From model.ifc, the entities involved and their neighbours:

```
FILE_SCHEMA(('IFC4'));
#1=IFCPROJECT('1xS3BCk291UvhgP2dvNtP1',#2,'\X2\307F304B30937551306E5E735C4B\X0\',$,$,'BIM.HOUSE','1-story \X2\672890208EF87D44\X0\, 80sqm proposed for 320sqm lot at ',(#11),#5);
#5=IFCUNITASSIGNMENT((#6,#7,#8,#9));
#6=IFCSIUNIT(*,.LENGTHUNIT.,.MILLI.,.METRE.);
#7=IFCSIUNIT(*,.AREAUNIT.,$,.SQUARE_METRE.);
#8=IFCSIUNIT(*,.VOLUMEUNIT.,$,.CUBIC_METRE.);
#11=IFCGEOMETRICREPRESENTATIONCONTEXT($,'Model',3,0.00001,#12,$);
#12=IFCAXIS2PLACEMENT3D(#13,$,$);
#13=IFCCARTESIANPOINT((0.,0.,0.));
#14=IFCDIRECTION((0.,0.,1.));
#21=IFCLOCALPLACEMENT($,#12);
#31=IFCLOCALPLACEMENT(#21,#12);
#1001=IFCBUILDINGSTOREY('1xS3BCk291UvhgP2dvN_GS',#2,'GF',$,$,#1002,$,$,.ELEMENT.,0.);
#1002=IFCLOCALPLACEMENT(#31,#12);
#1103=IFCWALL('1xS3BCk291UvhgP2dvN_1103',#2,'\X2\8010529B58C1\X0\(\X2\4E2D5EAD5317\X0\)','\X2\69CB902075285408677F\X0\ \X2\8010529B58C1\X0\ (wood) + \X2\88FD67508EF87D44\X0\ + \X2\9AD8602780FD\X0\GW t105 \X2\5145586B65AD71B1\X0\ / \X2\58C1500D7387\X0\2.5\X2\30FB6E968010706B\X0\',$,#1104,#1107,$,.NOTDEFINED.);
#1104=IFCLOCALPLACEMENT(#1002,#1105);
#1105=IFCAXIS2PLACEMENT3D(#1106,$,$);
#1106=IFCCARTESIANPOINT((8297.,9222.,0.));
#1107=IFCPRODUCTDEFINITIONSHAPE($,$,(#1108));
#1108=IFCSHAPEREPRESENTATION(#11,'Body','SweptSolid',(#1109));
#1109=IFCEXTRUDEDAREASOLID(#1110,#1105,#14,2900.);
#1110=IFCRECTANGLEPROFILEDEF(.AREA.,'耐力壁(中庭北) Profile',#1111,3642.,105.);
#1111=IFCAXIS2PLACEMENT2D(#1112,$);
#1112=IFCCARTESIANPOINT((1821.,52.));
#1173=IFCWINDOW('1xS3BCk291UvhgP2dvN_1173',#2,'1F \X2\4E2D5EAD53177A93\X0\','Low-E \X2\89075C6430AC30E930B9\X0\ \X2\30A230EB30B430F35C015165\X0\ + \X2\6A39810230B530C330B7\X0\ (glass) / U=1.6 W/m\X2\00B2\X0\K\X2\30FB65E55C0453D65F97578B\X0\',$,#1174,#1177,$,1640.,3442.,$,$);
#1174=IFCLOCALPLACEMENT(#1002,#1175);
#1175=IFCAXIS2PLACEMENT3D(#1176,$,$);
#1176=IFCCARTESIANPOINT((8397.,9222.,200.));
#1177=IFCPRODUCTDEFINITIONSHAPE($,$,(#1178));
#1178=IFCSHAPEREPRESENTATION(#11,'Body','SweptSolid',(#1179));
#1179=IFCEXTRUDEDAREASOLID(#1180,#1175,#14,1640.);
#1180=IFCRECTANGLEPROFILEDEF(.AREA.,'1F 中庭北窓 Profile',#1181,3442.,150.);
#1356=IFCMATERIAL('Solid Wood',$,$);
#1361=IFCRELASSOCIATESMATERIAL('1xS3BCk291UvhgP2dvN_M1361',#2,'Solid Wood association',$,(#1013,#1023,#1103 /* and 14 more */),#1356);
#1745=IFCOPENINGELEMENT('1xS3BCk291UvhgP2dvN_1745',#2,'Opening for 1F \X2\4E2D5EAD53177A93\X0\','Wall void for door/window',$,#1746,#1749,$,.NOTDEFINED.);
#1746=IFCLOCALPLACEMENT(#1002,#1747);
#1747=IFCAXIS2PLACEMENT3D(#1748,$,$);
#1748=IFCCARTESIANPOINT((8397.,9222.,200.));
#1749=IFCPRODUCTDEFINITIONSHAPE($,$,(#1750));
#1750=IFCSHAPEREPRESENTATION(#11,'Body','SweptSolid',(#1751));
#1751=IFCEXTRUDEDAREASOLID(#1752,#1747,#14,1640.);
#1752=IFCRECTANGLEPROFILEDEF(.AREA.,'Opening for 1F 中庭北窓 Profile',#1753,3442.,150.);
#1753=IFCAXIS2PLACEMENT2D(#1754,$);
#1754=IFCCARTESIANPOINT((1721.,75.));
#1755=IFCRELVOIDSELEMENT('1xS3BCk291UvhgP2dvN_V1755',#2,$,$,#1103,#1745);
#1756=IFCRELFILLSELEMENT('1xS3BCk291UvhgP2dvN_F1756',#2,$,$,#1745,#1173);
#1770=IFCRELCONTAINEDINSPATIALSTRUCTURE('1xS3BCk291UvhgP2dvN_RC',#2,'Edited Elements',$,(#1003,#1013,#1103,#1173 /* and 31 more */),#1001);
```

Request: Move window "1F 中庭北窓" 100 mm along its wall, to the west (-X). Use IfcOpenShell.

```python
import ifcopenshell
import ifcopenshell.api.geometry
import ifcopenshell.util.placement

model = ifcopenshell.open("model.ifc")

window = model.by_guid("1xS3BCk291UvhgP2dvN_1173")
opening = window.FillsVoids[0].RelatingOpeningElement
wall = opening.VoidsElements[0].RelatingBuildingElement

wall_matrix = ifcopenshell.util.placement.get_local_placement(wall.ObjectPlacement)
shift = wall_matrix[:3, 0] * -100.0
before = ifcopenshell.util.placement.get_local_placement(window.ObjectPlacement)[:3, 3].copy()

# The window is not placed relative to its opening, so move both.
for product in (opening, window):
    matrix = ifcopenshell.util.placement.get_local_placement(product.ObjectPlacement)
    matrix[:3, 3] += shift
    ifcopenshell.api.geometry.edit_object_placement(model, product=product, matrix=matrix, is_si=False)

after = ifcopenshell.util.placement.get_local_placement(window.ObjectPlacement)[:3, 3]
print("window moved by", (after - before).round(3) + 0.0)

model.write("model_rev.ifc")
```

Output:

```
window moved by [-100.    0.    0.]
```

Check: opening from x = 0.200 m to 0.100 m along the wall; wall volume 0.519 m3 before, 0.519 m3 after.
